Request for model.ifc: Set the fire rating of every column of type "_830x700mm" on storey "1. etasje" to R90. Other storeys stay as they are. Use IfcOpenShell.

First a look at what the model holds.

```python
import ifcopenshell
import ifcopenshell.util.element

model = ifcopenshell.open("model.ifc")
print(model.schema)
storey = next(s for s in model.by_type("IfcBuildingStorey") if s.Name == "1. etasje")
columns = [e for e in ifcopenshell.util.element.get_decomposition(storey) if e.is_a("IfcColumn")]
seen = {}
for e in columns:
    element_type = ifcopenshell.util.element.get_type(e)
    key = (element_type.Name if element_type != e and element_type else None, ifcopenshell.util.element.get_pset(e, "Pset_ColumnCommon", "FireRating"))
    seen[key] = seen.get(key, 0) + 1
for (name, value), count in sorted(seen.items(), key=str):
    print(count, "x", name, "|", value)
```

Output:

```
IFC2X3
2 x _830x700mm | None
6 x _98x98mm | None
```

```python
import ifcopenshell
import ifcopenshell.api.pset
import ifcopenshell.util.element

model = ifcopenshell.open("model.ifc")

storey = next(s for s in model.by_type("IfcBuildingStorey") if s.Name == "1. etasje")
columns = [e for e in ifcopenshell.util.element.get_decomposition(storey) if e.is_a("IfcColumn")]

count = 0
for e in columns:
    element_type = ifcopenshell.util.element.get_type(e)
    if element_type in (None, e) or element_type.Name != "_830x700mm":
        continue
    # add_pset returns the element's existing set when there is one.
    pset = ifcopenshell.api.pset.add_pset(model, product=e, name="Pset_ColumnCommon")
    ifcopenshell.api.pset.edit_pset(model, pset=pset, properties={"FireRating": "R90"})
    count += 1

print(count, "columns updated")

model.write("model_updated.ifc")
```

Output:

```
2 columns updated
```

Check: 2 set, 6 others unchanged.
